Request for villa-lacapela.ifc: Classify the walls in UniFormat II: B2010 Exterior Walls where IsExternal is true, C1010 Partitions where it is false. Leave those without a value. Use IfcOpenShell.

First a look at what the model holds.

```python
import ifcopenshell
import ifcopenshell.util.element

model = ifcopenshell.open("villa-lacapela.ifc")
print(model.schema)
print("classifications:", [c.Name for c in model.by_type("IfcClassification")])
values = [ifcopenshell.util.element.get_pset(e, "Pset_WallCommon", "IsExternal") for e in model.by_type("IfcWall")]
for value in (True, False, None):
    print("IsExternal", value, values.count(value))
```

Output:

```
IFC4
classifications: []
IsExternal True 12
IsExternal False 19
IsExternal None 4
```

```python
import ifcopenshell
import ifcopenshell.api.classification
import ifcopenshell.util.element

model = ifcopenshell.open("villa-lacapela.ifc")

system = ifcopenshell.api.classification.add_classification(model, classification="UniFormat II")

walls = model.by_type("IfcWall")
external = {e: ifcopenshell.util.element.get_pset(e, "Pset_WallCommon", "IsExternal") for e in walls}
for flag, code, name in ((True, "B2010", "Exterior Walls"), (False, "C1010", "Partitions")):
    products = [e for e in walls if external[e] is flag]
    ifcopenshell.api.classification.add_reference(
        model, products=products, classification=system, identification=code, name=name
    )
    print(code, len(products))

model.write("villa-lacapela-out.ifc")
```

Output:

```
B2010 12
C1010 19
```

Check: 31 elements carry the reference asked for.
